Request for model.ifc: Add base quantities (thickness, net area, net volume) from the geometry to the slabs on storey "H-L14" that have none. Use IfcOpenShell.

First a look at what the model holds.

```python
import ifcopenshell
import ifcopenshell.util.element
import ifcopenshell.util.unit

model = ifcopenshell.open("model.ifc")
print(model.schema)
for unit_type in ("LENGTHUNIT", "AREAUNIT", "VOLUMEUNIT"):
    print(unit_type, ifcopenshell.util.unit.calculate_unit_scale(model, unit_type))
storey = next(s for s in model.by_type("IfcBuildingStorey") if s.Name == "H-L14")
slabs = [e for e in ifcopenshell.util.element.get_decomposition(storey) if e.is_a("IfcSlab")]
for e in sorted(slabs, key=lambda e: e.id()):
    print(e.id(), e.is_a(), e.Name, list(ifcopenshell.util.element.get_psets(e, qtos_only=True)), sep=" | ")
```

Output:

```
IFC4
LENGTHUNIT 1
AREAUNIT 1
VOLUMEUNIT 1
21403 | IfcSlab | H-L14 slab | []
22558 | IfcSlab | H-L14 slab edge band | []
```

```python
import ifcopenshell
import ifcopenshell.api.pset
import ifcopenshell.geom
import ifcopenshell.util.element
import ifcopenshell.util.shape
import ifcopenshell.util.unit

model = ifcopenshell.open("model.ifc")
unit_scale = ifcopenshell.util.unit.calculate_unit_scale(model)
area_scale = ifcopenshell.util.unit.calculate_unit_scale(model, "AREAUNIT")
volume_scale = ifcopenshell.util.unit.calculate_unit_scale(model, "VOLUMEUNIT")
settings = ifcopenshell.geom.settings()

storey = next(s for s in model.by_type("IfcBuildingStorey") if s.Name == "H-L14")
slabs = [e for e in ifcopenshell.util.element.get_decomposition(storey) if e.is_a("IfcSlab")]

for e in sorted(slabs, key=lambda e: e.id()):
    if ifcopenshell.util.element.get_psets(e, qtos_only=True, should_inherit=False):
        continue
    # Geometry comes back in metres, in the element's own axes.
    shape = ifcopenshell.geom.create_shape(settings, e)
    values = {
        "Width": ifcopenshell.util.shape.get_z(shape.geometry) / unit_scale,
        "NetArea": ifcopenshell.util.shape.get_footprint_area(shape.geometry) / area_scale,
        "NetVolume": ifcopenshell.util.shape.get_volume(shape.geometry) / volume_scale,
    }
    qto = ifcopenshell.api.pset.add_qto(model, product=e, name="Qto_SlabBaseQuantities")
    ifcopenshell.api.pset.edit_qto(model, qto=qto, properties=values)
    print(e.id(), {k: round(v, 3) for k, v in values.items()})

model.write("model-out.ifc")
```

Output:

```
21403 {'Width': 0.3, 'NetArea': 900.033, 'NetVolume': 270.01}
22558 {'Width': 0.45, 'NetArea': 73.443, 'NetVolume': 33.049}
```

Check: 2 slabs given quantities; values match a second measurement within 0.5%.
